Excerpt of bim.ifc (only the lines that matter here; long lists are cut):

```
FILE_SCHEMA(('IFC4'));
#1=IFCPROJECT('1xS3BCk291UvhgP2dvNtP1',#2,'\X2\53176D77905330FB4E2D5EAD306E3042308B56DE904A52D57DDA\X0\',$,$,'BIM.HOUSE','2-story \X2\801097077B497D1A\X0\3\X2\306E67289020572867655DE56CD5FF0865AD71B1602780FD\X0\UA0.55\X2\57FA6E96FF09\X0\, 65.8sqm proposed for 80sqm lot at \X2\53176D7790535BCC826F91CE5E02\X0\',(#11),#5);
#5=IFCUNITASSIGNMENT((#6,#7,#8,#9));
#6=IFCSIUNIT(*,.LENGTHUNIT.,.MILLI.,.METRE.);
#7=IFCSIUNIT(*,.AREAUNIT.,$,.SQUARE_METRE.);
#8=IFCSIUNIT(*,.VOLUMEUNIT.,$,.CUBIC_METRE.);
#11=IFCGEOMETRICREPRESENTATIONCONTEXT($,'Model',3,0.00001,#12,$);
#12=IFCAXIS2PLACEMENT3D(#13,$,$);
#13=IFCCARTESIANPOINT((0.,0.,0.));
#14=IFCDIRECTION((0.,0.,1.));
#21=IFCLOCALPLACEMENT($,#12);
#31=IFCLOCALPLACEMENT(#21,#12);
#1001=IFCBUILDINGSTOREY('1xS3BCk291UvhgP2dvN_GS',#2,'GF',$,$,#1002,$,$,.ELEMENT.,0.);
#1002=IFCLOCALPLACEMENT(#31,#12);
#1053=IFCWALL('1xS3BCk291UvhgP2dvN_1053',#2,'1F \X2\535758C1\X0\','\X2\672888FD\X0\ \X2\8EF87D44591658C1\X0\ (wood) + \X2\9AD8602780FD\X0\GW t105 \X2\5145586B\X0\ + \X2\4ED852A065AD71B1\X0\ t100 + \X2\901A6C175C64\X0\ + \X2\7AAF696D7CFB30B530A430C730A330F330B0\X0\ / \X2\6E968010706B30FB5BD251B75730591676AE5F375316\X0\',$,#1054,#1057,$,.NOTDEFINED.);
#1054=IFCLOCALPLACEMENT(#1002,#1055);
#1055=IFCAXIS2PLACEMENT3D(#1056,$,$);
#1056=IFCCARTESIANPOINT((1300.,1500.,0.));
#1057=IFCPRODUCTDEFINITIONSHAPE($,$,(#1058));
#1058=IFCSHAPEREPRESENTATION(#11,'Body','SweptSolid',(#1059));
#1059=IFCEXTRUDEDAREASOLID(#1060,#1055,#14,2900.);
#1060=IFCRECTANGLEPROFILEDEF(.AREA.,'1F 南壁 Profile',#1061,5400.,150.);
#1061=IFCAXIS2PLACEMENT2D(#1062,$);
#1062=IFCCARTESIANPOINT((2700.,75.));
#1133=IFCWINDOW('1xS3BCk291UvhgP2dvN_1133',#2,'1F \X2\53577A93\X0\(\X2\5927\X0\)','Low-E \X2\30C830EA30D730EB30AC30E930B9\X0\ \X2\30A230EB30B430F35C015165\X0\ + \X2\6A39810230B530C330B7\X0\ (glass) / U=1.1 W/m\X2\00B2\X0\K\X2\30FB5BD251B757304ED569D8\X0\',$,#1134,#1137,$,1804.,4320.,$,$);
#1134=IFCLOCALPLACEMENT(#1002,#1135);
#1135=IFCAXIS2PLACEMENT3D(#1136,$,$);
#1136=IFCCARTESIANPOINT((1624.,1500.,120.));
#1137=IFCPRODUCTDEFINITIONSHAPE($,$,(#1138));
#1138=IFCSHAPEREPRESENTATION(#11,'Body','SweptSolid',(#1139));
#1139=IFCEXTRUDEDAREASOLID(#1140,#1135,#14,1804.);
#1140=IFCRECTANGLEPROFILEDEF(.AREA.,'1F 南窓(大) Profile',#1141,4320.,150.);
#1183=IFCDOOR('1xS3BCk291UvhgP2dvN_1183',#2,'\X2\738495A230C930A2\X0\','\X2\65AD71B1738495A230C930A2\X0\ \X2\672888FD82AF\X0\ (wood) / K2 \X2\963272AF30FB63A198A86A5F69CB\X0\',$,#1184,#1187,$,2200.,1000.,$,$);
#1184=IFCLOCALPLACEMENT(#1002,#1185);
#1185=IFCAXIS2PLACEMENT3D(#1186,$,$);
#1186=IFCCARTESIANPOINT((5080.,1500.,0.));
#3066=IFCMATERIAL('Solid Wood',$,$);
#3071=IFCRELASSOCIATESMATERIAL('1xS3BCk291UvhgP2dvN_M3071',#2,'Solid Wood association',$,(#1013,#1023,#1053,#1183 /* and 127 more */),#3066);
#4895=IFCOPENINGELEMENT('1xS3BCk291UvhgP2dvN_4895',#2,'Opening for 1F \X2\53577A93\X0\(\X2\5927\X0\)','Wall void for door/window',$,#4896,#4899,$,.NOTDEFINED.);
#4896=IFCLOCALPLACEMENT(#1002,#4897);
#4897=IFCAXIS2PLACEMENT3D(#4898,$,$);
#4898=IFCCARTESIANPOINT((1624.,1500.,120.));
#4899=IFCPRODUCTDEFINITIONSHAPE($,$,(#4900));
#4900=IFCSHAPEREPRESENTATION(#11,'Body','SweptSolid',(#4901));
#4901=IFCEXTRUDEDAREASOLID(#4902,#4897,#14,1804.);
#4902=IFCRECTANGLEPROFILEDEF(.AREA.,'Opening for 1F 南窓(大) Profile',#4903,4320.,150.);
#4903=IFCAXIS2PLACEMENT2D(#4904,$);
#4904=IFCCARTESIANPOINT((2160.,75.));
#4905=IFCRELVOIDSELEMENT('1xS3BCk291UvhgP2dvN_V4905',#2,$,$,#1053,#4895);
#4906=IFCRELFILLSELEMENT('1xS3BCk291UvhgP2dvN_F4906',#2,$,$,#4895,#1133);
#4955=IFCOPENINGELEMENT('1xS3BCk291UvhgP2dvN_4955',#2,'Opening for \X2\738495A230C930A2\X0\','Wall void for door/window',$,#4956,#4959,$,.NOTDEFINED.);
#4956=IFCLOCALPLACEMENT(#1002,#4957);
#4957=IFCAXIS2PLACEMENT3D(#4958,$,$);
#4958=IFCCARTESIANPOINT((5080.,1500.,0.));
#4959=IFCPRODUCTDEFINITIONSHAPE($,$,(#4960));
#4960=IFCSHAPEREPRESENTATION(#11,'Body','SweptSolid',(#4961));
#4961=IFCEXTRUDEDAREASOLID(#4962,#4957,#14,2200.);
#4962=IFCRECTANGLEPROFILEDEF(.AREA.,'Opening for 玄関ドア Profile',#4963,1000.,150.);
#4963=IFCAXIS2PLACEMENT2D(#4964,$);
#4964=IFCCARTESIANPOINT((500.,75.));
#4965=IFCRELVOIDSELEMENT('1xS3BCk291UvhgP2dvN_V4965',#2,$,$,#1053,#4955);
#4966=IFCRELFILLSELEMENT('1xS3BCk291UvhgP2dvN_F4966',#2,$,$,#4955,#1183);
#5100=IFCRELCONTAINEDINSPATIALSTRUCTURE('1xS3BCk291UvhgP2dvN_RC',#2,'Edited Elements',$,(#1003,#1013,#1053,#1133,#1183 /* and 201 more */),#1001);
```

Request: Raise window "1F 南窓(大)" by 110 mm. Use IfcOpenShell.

```python
import numpy as np
import ifcopenshell
import ifcopenshell.api.geometry
import ifcopenshell.util.placement
import ifcopenshell.util.unit

model = ifcopenshell.open("bim.ifc")
unit_scale = ifcopenshell.util.unit.calculate_unit_scale(model)

window = model.by_id(1133)
opening = window.FillsVoids[0].RelatingOpeningElement
dz = 0.11 / unit_scale

shift = np.array([0.0, 0.0, dz])
# The window is not placed relative to its opening, so move both.
for product in (opening, window):
    matrix = ifcopenshell.util.placement.get_local_placement(product.ObjectPlacement)
    matrix[:3, 3] += shift
    ifcopenshell.api.geometry.edit_object_placement(model, product=product, matrix=matrix, is_si=False)

print(f"moved by {dz * unit_scale:+.3f} m")

model.write("bim_updated.ifc")
```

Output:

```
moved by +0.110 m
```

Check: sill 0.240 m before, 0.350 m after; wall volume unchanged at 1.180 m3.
